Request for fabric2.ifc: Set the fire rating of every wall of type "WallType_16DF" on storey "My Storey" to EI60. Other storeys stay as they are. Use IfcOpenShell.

First a look at what the model holds.

```python
import ifcopenshell
import ifcopenshell.util.element

model = ifcopenshell.open("fabric2.ifc")
print(model.schema)
storey = next(s for s in model.by_type("IfcBuildingStorey") if s.Name == "My Storey")
walls = [e for e in ifcopenshell.util.element.get_decomposition(storey) if e.is_a("IfcWall")]
seen = {}
for e in walls:
    element_type = ifcopenshell.util.element.get_type(e)
    key = (element_type.Name if element_type != e and element_type else None, ifcopenshell.util.element.get_pset(e, "Pset_WallCommon", "FireRating"))
    seen[key] = seen.get(key, 0) + 1
for (name, value), count in sorted(seen.items(), key=str):
    print(count, "x", name, "|", value)
```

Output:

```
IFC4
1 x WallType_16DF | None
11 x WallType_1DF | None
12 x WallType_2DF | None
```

```python
import ifcopenshell
import ifcopenshell.api.pset
import ifcopenshell.util.element

model = ifcopenshell.open("fabric2.ifc")

storey = next(s for s in model.by_type("IfcBuildingStorey") if s.Name == "My Storey")
walls = [e for e in ifcopenshell.util.element.get_decomposition(storey) if e.is_a("IfcWall")]

count = 0
for e in walls:
    element_type = ifcopenshell.util.element.get_type(e)
    if element_type in (None, e) or element_type.Name != "WallType_16DF":
        continue
    # add_pset returns the element's existing set when there is one.
    pset = ifcopenshell.api.pset.add_pset(model, product=e, name="Pset_WallCommon")
    ifcopenshell.api.pset.edit_pset(model, pset=pset, properties={"FireRating": "EI60"})
    count += 1

print(count, "walls updated")

model.write("fabric2-out.ifc")
```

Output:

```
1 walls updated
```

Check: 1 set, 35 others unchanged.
